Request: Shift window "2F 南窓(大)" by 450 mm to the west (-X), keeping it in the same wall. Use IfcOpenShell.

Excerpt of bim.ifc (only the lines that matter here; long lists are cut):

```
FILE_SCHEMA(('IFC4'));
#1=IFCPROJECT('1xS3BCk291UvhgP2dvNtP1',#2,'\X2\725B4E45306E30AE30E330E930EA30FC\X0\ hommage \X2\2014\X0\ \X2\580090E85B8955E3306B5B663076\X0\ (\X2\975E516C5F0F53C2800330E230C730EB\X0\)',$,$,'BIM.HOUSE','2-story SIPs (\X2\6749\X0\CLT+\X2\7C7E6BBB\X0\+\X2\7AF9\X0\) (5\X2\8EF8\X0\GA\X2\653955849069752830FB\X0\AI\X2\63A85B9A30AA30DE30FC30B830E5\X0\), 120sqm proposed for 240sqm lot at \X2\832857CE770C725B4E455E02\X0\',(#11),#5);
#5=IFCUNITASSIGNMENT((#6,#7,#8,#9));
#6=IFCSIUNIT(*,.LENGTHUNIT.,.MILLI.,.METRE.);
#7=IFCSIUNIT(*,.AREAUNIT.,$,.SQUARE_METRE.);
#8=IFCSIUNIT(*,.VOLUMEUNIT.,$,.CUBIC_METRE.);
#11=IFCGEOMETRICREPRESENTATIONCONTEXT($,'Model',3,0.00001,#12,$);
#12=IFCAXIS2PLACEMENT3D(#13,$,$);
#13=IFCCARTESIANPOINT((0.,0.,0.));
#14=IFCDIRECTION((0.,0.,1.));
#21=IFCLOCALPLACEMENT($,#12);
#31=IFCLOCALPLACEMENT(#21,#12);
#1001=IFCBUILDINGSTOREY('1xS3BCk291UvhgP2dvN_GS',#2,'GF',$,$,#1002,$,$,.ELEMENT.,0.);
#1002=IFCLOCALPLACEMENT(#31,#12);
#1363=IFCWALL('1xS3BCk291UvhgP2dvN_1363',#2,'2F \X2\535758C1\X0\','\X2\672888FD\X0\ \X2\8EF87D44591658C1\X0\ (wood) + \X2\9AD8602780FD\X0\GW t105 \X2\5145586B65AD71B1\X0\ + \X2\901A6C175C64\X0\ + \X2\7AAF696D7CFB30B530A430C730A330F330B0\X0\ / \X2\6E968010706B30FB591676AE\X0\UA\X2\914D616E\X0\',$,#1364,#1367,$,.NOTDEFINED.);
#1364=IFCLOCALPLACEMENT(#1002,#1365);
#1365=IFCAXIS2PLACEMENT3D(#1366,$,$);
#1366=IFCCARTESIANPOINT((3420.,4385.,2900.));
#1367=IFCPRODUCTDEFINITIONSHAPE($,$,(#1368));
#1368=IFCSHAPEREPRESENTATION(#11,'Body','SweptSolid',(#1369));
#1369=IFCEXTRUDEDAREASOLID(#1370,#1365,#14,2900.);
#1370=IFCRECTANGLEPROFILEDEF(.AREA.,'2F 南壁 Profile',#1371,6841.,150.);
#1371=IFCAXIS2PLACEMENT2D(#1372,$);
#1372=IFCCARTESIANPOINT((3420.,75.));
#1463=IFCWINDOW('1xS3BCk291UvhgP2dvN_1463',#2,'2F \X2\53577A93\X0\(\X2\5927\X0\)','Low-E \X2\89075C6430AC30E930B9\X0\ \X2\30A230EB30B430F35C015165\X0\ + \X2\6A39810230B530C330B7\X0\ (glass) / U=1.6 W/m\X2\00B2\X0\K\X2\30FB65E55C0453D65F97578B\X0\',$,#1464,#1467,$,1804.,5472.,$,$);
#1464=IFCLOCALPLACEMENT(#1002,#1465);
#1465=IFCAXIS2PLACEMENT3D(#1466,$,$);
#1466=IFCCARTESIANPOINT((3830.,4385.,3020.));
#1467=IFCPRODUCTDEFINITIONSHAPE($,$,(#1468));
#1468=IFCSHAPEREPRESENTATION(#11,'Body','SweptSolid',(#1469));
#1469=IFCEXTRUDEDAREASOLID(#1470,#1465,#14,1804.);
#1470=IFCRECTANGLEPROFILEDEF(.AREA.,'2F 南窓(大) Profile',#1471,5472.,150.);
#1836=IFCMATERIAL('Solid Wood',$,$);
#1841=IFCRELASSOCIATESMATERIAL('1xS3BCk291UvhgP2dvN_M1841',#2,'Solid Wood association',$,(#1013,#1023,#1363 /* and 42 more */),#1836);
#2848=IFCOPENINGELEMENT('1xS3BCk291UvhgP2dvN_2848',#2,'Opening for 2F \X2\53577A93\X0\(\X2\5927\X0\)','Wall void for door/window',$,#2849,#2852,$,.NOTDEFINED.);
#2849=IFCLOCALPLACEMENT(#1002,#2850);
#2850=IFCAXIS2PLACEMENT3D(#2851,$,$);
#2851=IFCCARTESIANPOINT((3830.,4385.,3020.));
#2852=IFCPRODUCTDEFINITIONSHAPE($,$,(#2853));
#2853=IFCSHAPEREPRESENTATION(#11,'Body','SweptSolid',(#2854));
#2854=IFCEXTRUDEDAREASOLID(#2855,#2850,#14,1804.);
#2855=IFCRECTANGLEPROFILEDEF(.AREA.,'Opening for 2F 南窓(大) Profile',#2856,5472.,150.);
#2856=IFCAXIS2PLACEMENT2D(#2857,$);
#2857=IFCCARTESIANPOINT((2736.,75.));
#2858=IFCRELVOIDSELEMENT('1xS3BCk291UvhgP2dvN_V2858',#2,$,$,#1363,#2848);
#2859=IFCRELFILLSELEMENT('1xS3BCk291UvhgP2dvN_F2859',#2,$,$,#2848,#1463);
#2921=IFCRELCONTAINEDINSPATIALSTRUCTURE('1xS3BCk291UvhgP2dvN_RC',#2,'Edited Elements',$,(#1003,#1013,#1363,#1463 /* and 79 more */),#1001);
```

```python
import ifcopenshell
import ifcopenshell.api.geometry
import ifcopenshell.util.placement

model = ifcopenshell.open("bim.ifc")

window = model.by_id(1463)
opening = window.FillsVoids[0].RelatingOpeningElement
wall = opening.VoidsElements[0].RelatingBuildingElement

wall_matrix = ifcopenshell.util.placement.get_local_placement(wall.ObjectPlacement)
shift = wall_matrix[:3, 0] * -450.0
before = ifcopenshell.util.placement.get_local_placement(window.ObjectPlacement)[:3, 3].copy()

# The window is not placed relative to its opening, so move both.
for product in (opening, window):
    matrix = ifcopenshell.util.placement.get_local_placement(product.ObjectPlacement)
    matrix[:3, 3] += shift
    ifcopenshell.api.geometry.edit_object_placement(model, product=product, matrix=matrix, is_si=False)

after = ifcopenshell.util.placement.get_local_placement(window.ObjectPlacement)[:3, 3]
print("window moved by", (after - before).round(3) + 0.0)

model.write("bim_rev.ifc")
```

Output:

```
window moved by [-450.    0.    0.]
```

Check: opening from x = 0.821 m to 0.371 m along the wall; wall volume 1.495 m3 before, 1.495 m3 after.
